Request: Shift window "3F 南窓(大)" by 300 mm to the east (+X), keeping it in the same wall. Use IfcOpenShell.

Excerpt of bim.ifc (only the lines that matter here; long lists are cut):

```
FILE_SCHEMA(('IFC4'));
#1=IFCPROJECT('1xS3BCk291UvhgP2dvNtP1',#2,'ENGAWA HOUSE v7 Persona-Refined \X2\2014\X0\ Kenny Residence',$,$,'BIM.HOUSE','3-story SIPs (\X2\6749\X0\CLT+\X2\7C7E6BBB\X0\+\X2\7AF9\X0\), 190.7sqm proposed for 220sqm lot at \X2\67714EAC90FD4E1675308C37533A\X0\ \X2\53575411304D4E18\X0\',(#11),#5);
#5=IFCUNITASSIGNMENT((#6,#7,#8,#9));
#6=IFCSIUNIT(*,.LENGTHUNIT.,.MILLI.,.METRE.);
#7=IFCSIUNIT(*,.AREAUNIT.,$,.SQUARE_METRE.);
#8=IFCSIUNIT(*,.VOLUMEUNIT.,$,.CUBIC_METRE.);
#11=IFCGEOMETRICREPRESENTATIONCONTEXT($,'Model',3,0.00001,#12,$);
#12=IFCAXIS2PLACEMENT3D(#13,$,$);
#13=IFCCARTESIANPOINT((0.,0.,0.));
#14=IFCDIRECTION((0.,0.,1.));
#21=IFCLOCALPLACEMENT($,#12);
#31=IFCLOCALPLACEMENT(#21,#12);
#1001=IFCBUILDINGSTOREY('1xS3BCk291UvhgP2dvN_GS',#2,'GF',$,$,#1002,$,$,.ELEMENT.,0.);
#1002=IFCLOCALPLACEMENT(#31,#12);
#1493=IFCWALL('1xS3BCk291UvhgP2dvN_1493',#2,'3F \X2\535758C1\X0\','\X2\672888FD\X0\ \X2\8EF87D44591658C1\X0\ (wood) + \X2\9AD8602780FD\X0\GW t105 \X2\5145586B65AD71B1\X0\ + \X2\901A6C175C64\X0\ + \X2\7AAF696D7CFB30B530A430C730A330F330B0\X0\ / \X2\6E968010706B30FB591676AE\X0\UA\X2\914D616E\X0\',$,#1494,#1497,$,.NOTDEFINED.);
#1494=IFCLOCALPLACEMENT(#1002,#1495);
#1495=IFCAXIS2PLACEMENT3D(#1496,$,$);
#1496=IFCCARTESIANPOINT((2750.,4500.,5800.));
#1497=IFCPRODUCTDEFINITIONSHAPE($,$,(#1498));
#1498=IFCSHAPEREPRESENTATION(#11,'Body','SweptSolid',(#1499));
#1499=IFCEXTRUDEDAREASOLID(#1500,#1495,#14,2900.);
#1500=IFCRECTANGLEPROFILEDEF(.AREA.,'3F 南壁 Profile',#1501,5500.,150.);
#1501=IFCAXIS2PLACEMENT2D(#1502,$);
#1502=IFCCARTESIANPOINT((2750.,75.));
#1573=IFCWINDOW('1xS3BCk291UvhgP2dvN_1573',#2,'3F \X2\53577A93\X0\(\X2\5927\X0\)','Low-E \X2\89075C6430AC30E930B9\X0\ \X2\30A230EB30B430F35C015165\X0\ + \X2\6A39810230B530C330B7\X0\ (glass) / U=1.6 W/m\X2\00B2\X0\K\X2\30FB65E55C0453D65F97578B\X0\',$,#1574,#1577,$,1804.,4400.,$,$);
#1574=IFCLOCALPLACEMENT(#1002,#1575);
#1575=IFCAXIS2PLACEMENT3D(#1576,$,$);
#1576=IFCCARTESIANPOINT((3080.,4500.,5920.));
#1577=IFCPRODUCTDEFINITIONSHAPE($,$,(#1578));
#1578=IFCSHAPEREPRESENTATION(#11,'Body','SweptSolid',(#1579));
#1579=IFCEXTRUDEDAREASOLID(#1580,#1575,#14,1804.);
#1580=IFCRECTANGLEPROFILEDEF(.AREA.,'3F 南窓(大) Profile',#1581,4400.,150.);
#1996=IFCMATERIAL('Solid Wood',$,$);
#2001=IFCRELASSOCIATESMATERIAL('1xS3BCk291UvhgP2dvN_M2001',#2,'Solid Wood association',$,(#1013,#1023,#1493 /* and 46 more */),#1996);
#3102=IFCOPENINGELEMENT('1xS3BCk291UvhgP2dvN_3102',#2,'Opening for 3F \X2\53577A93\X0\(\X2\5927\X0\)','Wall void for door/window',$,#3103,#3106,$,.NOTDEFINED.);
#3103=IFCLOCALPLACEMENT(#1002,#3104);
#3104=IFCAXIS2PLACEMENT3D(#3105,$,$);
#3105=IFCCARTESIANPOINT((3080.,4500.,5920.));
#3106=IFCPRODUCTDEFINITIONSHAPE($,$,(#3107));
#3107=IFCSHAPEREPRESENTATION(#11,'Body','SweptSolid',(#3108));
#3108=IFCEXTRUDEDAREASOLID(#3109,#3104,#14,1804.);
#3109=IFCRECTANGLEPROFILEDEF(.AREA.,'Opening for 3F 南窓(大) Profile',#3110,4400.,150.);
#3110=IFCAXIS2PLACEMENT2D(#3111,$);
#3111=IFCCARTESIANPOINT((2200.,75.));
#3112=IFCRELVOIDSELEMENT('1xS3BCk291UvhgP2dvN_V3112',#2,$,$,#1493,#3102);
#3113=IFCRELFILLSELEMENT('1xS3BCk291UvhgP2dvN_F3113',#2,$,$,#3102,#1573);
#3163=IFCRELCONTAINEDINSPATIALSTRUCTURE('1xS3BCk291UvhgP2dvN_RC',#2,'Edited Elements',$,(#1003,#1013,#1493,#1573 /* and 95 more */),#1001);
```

```python
import ifcopenshell
import ifcopenshell.api.geometry
import ifcopenshell.util.placement
import ifcopenshell.util.unit

model = ifcopenshell.open("bim.ifc")
unit_scale = ifcopenshell.util.unit.calculate_unit_scale(model)

window = model.by_guid("1xS3BCk291UvhgP2dvN_1573")
opening = window.FillsVoids[0].RelatingOpeningElement
wall = opening.VoidsElements[0].RelatingBuildingElement

wall_matrix = ifcopenshell.util.placement.get_local_placement(wall.ObjectPlacement)
shift = wall_matrix[:3, 0] * 0.3 / unit_scale
before = ifcopenshell.util.placement.get_local_placement(window.ObjectPlacement)[:3, 3].copy()

# The window is not placed relative to its opening, so move both.
for product in (opening, window):
    matrix = ifcopenshell.util.placement.get_local_placement(product.ObjectPlacement)
    matrix[:3, 3] += shift
    ifcopenshell.api.geometry.edit_object_placement(model, product=product, matrix=matrix, is_si=False)

after = ifcopenshell.util.placement.get_local_placement(window.ObjectPlacement)[:3, 3]
print("window moved by", (after - before).round(3) + 0.0)

model.write("bim_v2.ifc")
```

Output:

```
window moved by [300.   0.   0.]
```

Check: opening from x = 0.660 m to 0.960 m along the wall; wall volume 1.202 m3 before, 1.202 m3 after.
